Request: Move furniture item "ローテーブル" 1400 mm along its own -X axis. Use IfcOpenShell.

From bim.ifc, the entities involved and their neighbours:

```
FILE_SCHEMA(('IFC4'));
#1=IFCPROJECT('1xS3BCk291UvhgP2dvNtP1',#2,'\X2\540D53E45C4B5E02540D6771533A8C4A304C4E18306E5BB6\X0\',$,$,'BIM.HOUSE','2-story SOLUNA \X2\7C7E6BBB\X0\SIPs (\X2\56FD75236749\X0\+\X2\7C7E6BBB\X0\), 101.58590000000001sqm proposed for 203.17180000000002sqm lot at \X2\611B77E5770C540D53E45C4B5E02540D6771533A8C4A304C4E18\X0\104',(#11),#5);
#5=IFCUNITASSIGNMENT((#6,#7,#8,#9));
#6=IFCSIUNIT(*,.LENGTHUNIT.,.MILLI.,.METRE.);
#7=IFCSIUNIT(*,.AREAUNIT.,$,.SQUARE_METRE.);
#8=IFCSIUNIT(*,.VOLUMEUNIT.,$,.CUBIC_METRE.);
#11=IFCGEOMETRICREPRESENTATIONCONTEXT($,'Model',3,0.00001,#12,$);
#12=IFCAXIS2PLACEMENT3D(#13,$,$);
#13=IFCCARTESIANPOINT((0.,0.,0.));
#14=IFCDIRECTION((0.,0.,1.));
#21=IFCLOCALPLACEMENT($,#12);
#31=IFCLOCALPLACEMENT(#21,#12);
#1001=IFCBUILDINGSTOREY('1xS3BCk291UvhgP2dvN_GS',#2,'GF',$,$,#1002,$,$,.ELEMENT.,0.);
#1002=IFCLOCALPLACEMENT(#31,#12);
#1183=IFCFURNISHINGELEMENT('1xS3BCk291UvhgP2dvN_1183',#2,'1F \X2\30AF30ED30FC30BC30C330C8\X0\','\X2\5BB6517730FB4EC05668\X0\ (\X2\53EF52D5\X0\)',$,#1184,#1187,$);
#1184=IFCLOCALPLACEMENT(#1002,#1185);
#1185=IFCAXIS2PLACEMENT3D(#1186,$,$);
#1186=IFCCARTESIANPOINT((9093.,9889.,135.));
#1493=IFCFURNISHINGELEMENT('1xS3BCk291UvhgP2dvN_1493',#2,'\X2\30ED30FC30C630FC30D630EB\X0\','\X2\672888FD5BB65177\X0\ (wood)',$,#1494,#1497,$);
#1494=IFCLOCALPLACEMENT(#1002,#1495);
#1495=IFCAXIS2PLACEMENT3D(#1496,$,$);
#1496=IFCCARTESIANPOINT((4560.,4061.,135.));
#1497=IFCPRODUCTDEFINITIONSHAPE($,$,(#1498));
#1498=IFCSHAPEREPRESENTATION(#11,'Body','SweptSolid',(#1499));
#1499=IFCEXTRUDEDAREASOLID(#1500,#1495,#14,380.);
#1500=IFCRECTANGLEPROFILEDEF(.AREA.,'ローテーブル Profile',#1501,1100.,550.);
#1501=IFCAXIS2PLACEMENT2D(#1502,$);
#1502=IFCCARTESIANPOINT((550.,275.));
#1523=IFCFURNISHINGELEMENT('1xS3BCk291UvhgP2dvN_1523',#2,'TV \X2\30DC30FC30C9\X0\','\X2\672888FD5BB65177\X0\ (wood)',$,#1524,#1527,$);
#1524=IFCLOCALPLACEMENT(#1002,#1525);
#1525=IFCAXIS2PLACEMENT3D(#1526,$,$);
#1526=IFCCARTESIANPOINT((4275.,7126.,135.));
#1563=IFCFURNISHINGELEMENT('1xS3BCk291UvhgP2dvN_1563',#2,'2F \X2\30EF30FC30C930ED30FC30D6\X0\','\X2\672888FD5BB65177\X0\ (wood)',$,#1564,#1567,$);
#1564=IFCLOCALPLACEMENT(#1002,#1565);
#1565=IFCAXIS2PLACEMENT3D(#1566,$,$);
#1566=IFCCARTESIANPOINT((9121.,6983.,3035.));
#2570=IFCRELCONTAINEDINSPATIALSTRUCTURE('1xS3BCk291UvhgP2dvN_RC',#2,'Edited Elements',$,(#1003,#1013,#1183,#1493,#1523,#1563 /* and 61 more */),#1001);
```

```python
import ifcopenshell
import ifcopenshell.api.geometry
import ifcopenshell.util.placement

model = ifcopenshell.open("bim.ifc")

item = model.by_guid("1xS3BCk291UvhgP2dvN_1493")
matrix = ifcopenshell.util.placement.get_local_placement(item.ObjectPlacement)
matrix[:3, 3] -= matrix[:3, 0] * 1400.0
ifcopenshell.api.geometry.edit_object_placement(model, product=item, matrix=matrix, is_si=False)

print(ifcopenshell.util.placement.get_local_placement(item.ObjectPlacement).round(3) + 0.0)

model.write("bim_rev.ifc")
```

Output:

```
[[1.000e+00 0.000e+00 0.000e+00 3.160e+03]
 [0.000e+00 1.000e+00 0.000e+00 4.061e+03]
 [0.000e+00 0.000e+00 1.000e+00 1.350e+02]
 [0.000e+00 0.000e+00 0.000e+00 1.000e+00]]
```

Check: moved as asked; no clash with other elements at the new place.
